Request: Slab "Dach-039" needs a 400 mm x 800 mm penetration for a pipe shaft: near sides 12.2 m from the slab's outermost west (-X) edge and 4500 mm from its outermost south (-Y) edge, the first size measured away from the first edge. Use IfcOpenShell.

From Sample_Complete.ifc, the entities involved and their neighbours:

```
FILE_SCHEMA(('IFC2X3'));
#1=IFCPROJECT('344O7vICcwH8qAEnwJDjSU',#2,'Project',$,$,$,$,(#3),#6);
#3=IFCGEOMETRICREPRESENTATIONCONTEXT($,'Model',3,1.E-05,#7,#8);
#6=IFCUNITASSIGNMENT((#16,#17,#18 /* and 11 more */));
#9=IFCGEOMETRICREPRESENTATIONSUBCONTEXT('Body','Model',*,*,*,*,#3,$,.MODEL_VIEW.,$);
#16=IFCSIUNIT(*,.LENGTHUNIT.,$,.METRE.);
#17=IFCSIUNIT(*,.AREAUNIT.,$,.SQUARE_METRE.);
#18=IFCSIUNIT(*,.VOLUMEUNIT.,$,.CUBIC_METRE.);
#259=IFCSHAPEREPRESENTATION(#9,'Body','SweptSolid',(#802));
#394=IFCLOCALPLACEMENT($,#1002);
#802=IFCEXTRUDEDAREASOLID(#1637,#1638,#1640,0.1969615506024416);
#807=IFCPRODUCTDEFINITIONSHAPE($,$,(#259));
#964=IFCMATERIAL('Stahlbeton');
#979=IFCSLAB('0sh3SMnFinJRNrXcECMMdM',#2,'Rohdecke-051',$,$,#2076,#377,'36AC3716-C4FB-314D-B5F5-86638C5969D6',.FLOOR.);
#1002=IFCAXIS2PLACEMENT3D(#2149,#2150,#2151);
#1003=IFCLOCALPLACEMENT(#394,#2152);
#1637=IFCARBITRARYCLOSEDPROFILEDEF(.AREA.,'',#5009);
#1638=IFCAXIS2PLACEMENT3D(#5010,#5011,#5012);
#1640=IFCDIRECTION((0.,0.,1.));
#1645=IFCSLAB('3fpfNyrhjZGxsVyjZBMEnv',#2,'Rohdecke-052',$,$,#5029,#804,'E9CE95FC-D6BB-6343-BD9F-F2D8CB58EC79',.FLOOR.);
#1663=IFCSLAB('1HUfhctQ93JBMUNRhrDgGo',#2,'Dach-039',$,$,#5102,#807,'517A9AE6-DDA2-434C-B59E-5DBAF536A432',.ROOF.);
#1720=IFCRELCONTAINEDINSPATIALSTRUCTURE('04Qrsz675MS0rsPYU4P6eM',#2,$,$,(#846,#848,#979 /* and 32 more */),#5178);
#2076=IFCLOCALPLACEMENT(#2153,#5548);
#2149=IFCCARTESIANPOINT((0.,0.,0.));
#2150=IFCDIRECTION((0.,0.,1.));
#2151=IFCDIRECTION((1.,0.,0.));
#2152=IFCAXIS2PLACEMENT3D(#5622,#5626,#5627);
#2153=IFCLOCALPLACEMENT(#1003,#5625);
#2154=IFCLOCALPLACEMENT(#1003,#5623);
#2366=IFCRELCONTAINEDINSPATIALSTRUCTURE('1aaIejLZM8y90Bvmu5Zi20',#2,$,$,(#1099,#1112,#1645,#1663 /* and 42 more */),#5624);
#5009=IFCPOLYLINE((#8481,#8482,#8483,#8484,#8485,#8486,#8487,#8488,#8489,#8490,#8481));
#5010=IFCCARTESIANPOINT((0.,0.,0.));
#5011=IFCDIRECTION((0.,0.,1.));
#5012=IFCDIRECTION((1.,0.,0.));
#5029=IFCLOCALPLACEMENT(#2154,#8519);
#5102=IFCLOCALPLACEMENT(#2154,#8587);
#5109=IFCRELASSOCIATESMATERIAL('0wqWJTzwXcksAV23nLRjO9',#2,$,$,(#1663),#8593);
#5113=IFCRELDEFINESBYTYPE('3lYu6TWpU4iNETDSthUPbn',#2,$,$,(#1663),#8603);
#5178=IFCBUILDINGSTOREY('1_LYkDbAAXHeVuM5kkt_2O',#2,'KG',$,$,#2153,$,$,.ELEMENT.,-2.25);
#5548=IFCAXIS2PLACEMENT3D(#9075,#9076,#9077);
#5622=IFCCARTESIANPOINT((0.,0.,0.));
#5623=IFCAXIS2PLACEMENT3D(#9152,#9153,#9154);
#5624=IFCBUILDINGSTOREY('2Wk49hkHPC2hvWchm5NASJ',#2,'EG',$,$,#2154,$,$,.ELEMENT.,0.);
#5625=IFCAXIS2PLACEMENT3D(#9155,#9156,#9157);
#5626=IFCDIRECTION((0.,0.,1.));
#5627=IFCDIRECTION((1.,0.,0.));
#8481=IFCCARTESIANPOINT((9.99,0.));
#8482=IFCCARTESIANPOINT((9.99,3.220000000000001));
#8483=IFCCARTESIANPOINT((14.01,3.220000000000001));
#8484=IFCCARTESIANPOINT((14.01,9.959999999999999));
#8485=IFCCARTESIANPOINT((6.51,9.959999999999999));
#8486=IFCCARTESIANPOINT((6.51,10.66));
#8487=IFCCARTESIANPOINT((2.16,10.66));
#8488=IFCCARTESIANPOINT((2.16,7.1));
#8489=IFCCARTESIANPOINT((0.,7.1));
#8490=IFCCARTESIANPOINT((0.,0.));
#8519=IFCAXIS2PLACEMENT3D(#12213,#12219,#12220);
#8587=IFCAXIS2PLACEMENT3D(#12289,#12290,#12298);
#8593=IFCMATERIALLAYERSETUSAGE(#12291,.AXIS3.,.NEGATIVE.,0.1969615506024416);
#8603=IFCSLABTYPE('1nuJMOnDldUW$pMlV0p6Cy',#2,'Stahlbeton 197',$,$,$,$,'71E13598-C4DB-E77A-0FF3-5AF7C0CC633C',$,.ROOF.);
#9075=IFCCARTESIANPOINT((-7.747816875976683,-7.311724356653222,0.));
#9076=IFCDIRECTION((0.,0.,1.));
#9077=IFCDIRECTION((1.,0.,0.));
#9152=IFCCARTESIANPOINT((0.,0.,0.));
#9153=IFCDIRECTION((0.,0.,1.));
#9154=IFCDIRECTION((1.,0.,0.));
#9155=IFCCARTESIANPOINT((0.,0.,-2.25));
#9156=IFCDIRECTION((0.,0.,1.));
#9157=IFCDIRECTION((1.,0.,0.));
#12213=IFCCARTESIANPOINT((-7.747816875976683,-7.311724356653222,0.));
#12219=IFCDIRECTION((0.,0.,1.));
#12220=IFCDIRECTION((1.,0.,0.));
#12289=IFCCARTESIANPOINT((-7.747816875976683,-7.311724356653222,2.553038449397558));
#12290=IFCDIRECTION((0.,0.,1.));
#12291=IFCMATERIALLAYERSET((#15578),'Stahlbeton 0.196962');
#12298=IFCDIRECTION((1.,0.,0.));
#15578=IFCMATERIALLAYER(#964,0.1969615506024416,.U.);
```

```python
import numpy as np
import ifcopenshell
import ifcopenshell.api.feature
import ifcopenshell.api.geometry
import ifcopenshell.api.root
import ifcopenshell.geom
import ifcopenshell.util.placement
import ifcopenshell.util.representation
import ifcopenshell.util.shape
import ifcopenshell.util.unit

model = ifcopenshell.open("Sample_Complete.ifc")
unit_scale = ifcopenshell.util.unit.calculate_unit_scale(model)
settings = ifcopenshell.geom.settings()


def volume(element):
    """Net volume in cubic metres, openings subtracted."""
    shape = ifcopenshell.geom.create_shape(settings, element)
    return ifcopenshell.util.shape.get_volume(shape.geometry)


slab = model.by_id(1663)
before = volume(slab)

# Extent in the slab's own axes, in metres. The edges named are its -X and -Y sides.
slab_shape = ifcopenshell.geom.create_shape(settings, slab)
vertices = ifcopenshell.util.shape.get_vertices(slab_shape.geometry)
x_min, y_min, bottom = vertices.min(axis=0)
top = vertices[:, 2].max()

opening = ifcopenshell.api.root.create_entity(model, ifc_class="IfcOpeningElement", name="Pipe shaft opening")
context = ifcopenshell.util.representation.get_context(model, "Model", "Body", "MODEL_VIEW")
width, depth = 0.4, 0.8
outline = [(0.0, 0.0), (width, 0.0), (width, depth), (0.0, depth), (0.0, 0.0)]
# Overshoot both faces by 50 mm so the cut is clean.
shape = ifcopenshell.api.geometry.add_slab_representation(
    model, context=context, depth=top - bottom + 0.1, polyline=outline
)
ifcopenshell.api.geometry.assign_representation(model, product=opening, representation=shape)

matrix = ifcopenshell.util.placement.get_local_placement(slab.ObjectPlacement)
matrix[:, 3] = matrix @ np.append(np.array([x_min + 12.2, y_min + 4.5, bottom - 0.05]) / unit_scale, 1.0)
ifcopenshell.api.geometry.edit_object_placement(model, product=opening, matrix=matrix, is_si=False)
ifcopenshell.api.feature.add_feature(model, feature=opening, element=slab)

after = volume(slab)

print(f"slab volume {before:.3f} -> {after:.3f} m3")

model.write("Sample_Complete_rev.ifc")
```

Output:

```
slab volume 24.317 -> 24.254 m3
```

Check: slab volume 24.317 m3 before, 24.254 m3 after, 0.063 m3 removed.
